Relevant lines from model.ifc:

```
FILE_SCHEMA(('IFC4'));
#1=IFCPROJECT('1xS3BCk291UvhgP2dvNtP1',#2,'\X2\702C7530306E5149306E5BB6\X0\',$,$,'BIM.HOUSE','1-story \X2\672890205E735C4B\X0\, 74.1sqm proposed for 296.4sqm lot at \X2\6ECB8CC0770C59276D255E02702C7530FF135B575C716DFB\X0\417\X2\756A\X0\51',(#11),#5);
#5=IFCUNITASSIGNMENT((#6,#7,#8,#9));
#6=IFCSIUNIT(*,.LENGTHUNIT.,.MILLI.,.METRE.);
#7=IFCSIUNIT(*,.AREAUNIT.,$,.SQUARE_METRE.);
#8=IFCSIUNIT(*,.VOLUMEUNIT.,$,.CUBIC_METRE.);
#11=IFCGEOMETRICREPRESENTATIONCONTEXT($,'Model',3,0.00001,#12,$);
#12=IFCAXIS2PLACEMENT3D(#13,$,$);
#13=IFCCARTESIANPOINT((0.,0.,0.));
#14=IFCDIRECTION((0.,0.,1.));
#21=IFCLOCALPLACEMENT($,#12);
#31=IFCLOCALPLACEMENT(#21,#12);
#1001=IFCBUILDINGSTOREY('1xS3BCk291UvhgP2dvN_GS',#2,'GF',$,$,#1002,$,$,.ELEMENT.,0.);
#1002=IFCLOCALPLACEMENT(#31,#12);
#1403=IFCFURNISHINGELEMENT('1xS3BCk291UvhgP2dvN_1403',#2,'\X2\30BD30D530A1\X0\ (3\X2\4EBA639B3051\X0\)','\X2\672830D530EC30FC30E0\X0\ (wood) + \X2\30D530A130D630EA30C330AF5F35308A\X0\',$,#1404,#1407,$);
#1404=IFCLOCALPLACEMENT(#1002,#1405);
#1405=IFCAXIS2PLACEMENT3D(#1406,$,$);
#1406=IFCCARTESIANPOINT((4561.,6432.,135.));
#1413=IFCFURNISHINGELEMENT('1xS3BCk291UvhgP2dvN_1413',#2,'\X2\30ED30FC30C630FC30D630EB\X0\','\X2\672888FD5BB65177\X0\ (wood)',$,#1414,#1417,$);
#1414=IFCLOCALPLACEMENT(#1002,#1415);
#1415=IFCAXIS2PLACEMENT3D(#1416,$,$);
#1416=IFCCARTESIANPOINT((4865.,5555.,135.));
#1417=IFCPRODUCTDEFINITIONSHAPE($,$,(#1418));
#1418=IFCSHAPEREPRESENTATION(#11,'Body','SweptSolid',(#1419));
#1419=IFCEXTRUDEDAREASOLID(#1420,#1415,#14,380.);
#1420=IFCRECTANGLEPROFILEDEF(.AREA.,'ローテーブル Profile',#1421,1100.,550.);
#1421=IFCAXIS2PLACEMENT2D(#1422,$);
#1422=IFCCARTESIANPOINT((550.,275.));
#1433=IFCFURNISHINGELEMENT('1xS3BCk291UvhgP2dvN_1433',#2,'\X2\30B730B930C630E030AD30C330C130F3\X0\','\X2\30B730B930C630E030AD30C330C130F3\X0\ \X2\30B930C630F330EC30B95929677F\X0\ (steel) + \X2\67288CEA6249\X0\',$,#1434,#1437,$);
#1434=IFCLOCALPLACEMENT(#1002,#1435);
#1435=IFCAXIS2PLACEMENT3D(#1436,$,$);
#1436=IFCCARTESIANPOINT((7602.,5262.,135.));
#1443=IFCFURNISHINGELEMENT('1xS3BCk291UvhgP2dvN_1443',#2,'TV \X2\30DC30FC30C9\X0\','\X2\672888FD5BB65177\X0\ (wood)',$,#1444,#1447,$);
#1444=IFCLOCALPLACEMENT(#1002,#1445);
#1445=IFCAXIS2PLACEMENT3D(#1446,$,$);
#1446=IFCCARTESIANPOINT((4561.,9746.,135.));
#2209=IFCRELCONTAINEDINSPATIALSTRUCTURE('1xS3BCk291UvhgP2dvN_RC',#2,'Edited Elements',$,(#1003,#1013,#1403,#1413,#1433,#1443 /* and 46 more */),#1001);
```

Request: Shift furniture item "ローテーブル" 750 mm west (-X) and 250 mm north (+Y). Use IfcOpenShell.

```python
import ifcopenshell
import ifcopenshell.api.geometry
import ifcopenshell.util.placement
import ifcopenshell.util.unit

model = ifcopenshell.open("model.ifc")
unit_scale = ifcopenshell.util.unit.calculate_unit_scale(model)

item = model.by_id(1413)
matrix = ifcopenshell.util.placement.get_local_placement(item.ObjectPlacement)
matrix[0, 3] -= 0.75 / unit_scale
matrix[1, 3] += 0.25 / unit_scale
ifcopenshell.api.geometry.edit_object_placement(model, product=item, matrix=matrix, is_si=False)

print(ifcopenshell.util.placement.get_local_placement(item.ObjectPlacement).round(3) + 0.0)

model.write("model_edited.ifc")
```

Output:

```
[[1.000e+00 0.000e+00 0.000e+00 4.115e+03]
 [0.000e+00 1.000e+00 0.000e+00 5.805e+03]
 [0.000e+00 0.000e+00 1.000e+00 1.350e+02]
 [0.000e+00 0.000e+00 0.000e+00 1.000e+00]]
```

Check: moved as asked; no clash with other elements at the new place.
